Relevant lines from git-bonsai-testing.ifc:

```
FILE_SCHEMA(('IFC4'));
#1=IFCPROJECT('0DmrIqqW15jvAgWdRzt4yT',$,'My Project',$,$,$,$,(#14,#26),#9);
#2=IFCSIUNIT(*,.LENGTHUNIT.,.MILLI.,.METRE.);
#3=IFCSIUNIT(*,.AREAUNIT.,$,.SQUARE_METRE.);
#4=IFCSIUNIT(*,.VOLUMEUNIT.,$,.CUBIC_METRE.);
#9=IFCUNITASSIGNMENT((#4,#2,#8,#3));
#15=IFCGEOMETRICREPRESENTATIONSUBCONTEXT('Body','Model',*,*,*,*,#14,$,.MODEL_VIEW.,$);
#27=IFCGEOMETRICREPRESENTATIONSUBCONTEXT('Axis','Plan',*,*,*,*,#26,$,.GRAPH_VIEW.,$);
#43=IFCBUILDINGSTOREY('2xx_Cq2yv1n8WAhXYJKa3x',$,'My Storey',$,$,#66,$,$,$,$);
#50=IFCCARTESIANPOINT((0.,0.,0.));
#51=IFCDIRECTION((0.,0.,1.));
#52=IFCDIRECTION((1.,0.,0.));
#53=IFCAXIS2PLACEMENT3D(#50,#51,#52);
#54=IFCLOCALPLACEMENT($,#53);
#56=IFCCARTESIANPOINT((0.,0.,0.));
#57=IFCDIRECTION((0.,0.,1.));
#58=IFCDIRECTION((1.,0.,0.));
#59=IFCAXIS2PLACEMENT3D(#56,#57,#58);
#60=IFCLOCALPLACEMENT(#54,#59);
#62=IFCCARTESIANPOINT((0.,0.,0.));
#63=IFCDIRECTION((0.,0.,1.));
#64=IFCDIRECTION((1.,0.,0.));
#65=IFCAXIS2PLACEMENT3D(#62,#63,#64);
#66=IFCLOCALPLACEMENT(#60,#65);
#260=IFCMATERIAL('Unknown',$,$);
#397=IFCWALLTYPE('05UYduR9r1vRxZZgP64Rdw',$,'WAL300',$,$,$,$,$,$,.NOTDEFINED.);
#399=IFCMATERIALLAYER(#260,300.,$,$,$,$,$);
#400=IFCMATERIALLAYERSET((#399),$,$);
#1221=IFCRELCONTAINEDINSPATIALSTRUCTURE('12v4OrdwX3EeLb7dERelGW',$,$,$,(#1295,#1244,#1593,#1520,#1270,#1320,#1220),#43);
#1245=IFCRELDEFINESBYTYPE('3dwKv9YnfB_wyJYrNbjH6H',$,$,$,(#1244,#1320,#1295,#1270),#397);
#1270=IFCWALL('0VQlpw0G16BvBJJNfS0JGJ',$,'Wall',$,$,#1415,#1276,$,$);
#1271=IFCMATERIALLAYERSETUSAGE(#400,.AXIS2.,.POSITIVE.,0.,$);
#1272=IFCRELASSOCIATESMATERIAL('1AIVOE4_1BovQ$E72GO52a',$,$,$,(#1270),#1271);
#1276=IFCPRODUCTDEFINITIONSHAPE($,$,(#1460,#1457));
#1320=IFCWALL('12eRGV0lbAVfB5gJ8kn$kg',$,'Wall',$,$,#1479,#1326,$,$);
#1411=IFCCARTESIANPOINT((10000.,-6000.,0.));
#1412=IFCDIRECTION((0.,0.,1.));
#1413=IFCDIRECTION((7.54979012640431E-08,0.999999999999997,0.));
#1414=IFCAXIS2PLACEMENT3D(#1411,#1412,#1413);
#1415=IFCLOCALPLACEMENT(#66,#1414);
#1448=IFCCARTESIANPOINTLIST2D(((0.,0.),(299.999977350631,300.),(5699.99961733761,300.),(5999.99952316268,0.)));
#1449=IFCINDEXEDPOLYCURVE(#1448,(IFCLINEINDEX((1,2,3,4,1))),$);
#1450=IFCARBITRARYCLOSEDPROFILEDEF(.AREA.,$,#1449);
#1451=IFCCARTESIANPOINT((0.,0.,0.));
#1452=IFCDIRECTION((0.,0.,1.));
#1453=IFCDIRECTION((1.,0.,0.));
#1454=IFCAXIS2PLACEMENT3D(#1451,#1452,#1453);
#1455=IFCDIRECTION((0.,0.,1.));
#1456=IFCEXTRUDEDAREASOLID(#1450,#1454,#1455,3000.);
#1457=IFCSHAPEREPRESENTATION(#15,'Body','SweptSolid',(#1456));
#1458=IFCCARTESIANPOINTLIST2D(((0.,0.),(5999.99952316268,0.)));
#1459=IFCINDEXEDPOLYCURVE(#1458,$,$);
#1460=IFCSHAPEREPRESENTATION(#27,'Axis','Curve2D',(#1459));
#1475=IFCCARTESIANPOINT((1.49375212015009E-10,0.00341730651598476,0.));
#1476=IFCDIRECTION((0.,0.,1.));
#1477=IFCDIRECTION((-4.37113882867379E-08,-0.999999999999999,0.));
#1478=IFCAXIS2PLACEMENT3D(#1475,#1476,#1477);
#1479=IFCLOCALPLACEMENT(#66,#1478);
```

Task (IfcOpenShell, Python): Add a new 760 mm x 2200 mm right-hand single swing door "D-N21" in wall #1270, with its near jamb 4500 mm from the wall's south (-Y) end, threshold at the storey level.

```python
import numpy as np
import ifcopenshell
import ifcopenshell.api.feature
import ifcopenshell.api.geometry
import ifcopenshell.api.root
import ifcopenshell.api.spatial
import ifcopenshell.geom
import ifcopenshell.util.element
import ifcopenshell.util.placement
import ifcopenshell.util.representation
import ifcopenshell.util.shape
import ifcopenshell.util.unit

model = ifcopenshell.open("git-bonsai-testing.ifc")
unit_scale = ifcopenshell.util.unit.calculate_unit_scale(model)
settings = ifcopenshell.geom.settings()


def volume(element):
    """Net volume in cubic metres, openings subtracted."""
    shape = ifcopenshell.geom.create_shape(settings, element)
    return ifcopenshell.util.shape.get_volume(shape.geometry)


wall = model.by_guid("0VQlpw0G16BvBJJNfS0JGJ")
storey = ifcopenshell.util.element.get_container(wall, ifc_class="IfcBuildingStorey")
context = ifcopenshell.util.representation.get_context(model, "Model", "Body", "MODEL_VIEW")
before = volume(wall)

width, height, from_end, sill = 0.76, 2.2, 4.5, 0.0  # metres

# The wall runs along its own X axis, and the end named is its -X end.
wall_shape = ifcopenshell.geom.create_shape(settings, wall)
x, y, z = ifcopenshell.util.shape.get_vertices(wall_shape.geometry).T
start = x.min() + from_end
face, thickness = float(y.min()), float(y.max() - y.min())
wall_matrix = ifcopenshell.util.placement.get_local_placement(wall.ObjectPlacement)
level = ifcopenshell.util.placement.get_local_placement(storey.ObjectPlacement)[2, 3]


def in_wall(x, y):
    """Placement at x, y metres in the wall's axes, at sill height."""
    matrix = wall_matrix.copy()
    matrix[:, 3] = wall_matrix @ np.array([x / unit_scale, y / unit_scale, 0.0, 1.0])
    matrix[2, 3] = level + sill / unit_scale
    return matrix


# Opening: a box that overshoots both wall faces by 50 mm.
opening = ifcopenshell.api.root.create_entity(model, ifc_class="IfcOpeningElement", predefined_type="OPENING")
box = ifcopenshell.api.geometry.add_wall_representation(
    model, context=context, length=width, height=height, thickness=thickness + 0.1
)
ifcopenshell.api.geometry.assign_representation(model, product=opening, representation=box)
ifcopenshell.api.geometry.edit_object_placement(model, product=opening, matrix=in_wall(start, face - 0.05), is_si=False)
ifcopenshell.api.feature.add_feature(model, feature=opening, element=wall)

door = ifcopenshell.api.root.create_entity(model, ifc_class="IfcDoor", name="D-N21", predefined_type="DOOR")
door.OverallWidth, door.OverallHeight = width / unit_scale, height / unit_scale
door.OperationType = "SINGLE_SWING_RIGHT"
body = ifcopenshell.api.geometry.add_door_representation(
    model,
    context=context,
    overall_width=door.OverallWidth,
    overall_height=door.OverallHeight,
    operation_type="SINGLE_SWING_RIGHT",
    lining_properties={"LiningDepth": thickness / unit_scale, "ThresholdDepth": thickness / unit_scale},
)
ifcopenshell.api.geometry.assign_representation(model, product=door, representation=body)
ifcopenshell.api.spatial.assign_container(model, products=[door], relating_structure=storey)
ifcopenshell.api.feature.add_filling(model, opening=opening, element=door)

# The lining spans the wall, so the door starts at the wall face.
ifcopenshell.api.geometry.edit_object_placement(model, product=door, matrix=in_wall(start, face), is_si=False)

after = volume(wall)

print(f"wall volume {before:.3f} -> {after:.3f} m3")

model.write("git-bonsai-testing_updated.ifc")
```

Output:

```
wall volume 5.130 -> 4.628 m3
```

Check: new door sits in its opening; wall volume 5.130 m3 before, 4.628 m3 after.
